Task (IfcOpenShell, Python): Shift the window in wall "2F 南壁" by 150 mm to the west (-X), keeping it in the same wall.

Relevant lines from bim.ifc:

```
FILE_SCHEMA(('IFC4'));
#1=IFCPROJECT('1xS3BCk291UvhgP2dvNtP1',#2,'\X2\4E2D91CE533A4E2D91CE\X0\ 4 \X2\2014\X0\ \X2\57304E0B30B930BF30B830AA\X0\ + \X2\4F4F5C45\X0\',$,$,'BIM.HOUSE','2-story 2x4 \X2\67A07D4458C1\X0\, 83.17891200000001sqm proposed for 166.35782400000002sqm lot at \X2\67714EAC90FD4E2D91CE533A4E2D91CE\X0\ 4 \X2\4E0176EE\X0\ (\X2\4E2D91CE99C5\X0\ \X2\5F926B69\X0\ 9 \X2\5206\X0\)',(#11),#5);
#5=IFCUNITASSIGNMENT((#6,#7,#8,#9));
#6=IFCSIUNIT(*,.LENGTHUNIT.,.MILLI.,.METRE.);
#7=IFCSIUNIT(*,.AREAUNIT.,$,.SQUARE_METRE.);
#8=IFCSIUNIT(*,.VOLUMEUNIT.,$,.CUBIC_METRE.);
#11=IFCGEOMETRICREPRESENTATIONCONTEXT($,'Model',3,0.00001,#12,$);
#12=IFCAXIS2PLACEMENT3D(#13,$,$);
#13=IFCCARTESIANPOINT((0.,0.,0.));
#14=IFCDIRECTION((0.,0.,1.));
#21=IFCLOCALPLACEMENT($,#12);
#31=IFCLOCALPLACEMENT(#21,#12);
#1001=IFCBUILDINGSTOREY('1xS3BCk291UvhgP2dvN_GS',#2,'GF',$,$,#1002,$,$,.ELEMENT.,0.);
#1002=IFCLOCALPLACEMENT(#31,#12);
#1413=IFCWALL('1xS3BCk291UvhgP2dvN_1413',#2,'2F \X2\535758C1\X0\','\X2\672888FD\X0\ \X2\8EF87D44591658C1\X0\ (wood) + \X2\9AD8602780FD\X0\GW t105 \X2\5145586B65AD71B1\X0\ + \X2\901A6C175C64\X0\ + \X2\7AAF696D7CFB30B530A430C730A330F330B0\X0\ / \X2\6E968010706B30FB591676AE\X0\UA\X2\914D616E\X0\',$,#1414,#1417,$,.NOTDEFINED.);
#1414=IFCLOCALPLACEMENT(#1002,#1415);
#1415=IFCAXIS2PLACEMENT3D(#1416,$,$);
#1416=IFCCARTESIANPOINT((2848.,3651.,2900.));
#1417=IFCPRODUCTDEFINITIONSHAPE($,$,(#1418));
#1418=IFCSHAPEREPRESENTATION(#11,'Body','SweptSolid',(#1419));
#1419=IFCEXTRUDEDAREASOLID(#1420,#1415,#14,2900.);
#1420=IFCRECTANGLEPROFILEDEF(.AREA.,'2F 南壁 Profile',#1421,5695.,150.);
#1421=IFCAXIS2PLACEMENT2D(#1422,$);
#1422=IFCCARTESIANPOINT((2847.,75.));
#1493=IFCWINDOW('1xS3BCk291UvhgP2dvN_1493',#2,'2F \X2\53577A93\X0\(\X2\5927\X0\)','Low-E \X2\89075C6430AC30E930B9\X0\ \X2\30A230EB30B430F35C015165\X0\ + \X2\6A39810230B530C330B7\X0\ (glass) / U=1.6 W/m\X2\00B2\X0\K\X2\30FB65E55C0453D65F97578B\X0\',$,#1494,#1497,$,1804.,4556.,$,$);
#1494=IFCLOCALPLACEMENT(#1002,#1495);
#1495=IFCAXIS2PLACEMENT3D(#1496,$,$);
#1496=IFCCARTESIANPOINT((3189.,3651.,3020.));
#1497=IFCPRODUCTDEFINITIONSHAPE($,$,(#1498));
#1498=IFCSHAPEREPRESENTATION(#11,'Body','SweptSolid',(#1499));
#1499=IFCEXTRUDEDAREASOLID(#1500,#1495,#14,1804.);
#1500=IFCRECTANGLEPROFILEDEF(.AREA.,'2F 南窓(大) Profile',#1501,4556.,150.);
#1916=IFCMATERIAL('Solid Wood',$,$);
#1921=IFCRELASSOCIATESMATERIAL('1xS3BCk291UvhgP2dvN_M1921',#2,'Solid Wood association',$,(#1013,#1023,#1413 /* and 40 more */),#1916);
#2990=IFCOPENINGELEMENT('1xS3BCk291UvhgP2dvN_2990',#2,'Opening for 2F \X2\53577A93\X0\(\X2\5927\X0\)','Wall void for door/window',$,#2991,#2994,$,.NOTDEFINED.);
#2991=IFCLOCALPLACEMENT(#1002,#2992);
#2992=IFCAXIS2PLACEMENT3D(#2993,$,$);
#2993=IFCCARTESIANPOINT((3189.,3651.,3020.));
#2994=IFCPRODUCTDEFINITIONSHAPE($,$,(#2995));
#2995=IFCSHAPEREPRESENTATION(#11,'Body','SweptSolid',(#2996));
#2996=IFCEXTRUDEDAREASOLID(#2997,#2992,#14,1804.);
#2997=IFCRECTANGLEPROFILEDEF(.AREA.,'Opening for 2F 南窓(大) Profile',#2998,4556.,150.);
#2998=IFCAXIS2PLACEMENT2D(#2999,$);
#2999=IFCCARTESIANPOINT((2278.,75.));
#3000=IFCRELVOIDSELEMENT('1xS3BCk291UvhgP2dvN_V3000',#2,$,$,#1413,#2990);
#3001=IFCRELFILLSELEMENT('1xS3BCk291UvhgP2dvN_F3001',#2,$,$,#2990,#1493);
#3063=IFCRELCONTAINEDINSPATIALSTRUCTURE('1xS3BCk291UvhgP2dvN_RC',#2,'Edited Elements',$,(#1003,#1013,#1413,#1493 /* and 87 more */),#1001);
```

```python
import ifcopenshell
import ifcopenshell.api.geometry
import ifcopenshell.util.placement

model = ifcopenshell.open("bim.ifc")

window = model.by_guid("1xS3BCk291UvhgP2dvN_1493")
opening = window.FillsVoids[0].RelatingOpeningElement
wall = opening.VoidsElements[0].RelatingBuildingElement

wall_matrix = ifcopenshell.util.placement.get_local_placement(wall.ObjectPlacement)
shift = wall_matrix[:3, 0] * -150.0
before = ifcopenshell.util.placement.get_local_placement(window.ObjectPlacement)[:3, 3].copy()

# The window is not placed relative to its opening, so move both.
for product in (opening, window):
    matrix = ifcopenshell.util.placement.get_local_placement(product.ObjectPlacement)
    matrix[:3, 3] += shift
    ifcopenshell.api.geometry.edit_object_placement(model, product=product, matrix=matrix, is_si=False)

after = ifcopenshell.util.placement.get_local_placement(window.ObjectPlacement)[:3, 3]
print("window moved by", (after - before).round(3) + 0.0)

model.write("bim_v2.ifc")
```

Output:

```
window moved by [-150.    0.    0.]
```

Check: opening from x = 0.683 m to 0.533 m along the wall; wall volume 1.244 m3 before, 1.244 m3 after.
